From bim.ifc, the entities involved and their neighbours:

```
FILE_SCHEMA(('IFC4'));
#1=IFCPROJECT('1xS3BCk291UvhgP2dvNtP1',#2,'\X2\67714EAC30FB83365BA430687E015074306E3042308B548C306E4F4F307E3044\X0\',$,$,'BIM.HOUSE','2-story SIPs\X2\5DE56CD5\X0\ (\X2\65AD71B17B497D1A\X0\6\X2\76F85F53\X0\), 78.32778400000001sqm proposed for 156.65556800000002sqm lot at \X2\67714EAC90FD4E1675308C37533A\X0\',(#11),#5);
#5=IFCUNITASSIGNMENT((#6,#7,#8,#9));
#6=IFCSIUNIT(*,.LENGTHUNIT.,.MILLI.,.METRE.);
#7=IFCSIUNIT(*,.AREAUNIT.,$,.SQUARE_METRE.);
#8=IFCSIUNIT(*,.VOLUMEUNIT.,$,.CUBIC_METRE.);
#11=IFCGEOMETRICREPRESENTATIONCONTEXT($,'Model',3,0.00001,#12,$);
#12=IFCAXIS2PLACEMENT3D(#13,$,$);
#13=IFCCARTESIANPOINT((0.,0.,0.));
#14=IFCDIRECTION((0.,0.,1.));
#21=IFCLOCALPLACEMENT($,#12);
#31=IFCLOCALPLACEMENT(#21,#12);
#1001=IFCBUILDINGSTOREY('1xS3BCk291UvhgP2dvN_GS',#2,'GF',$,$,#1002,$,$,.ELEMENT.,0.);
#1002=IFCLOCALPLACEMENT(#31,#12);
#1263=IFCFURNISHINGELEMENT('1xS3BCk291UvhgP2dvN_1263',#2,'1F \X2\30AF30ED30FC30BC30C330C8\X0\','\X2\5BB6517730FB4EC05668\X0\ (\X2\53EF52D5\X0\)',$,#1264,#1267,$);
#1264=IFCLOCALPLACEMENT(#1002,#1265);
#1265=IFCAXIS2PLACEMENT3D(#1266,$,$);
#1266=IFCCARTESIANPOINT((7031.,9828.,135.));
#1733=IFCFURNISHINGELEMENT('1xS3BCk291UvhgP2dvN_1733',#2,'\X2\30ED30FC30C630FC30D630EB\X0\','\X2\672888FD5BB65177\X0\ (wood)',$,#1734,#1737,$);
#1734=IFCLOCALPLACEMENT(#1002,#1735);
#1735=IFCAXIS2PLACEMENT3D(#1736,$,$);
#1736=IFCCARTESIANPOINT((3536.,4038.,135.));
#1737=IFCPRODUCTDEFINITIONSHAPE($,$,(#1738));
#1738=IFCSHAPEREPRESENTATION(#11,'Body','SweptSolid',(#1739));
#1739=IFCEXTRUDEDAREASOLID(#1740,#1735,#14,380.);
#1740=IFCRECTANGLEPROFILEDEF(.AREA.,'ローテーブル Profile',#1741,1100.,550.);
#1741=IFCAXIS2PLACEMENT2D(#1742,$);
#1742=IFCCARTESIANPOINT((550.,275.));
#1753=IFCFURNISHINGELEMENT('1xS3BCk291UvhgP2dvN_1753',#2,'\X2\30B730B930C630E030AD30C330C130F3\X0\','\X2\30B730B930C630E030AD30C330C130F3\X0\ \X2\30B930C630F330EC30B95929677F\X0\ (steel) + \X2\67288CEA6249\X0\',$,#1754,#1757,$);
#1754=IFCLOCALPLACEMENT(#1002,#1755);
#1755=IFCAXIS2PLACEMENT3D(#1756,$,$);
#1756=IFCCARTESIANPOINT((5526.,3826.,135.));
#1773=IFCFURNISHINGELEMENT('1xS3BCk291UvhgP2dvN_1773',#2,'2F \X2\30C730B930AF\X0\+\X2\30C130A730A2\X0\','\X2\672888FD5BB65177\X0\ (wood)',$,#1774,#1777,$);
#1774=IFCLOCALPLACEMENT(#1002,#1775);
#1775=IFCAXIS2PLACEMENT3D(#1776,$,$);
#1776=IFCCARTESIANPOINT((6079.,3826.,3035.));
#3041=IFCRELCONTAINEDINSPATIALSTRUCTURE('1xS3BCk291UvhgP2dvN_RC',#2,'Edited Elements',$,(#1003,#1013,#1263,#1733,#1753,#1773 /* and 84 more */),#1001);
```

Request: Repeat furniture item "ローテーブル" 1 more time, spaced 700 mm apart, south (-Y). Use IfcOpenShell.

```python
import numpy as np
import ifcopenshell
import ifcopenshell.api.geometry
import ifcopenshell.api.root
import ifcopenshell.util.element
import ifcopenshell.util.placement
import ifcopenshell.util.unit

model = ifcopenshell.open("bim.ifc")
unit_scale = ifcopenshell.util.unit.calculate_unit_scale(model)


def reuse_history(source, copy):
    """copy_class also copies each property set's owner history, people and application; keep the originals."""
    for rel in copy.IsDefinedBy:
        if rel.is_a("IfcRelDefinesByProperties") and (history := rel.RelatingPropertyDefinition.OwnerHistory):
            rel.RelatingPropertyDefinition.OwnerHistory = source.OwnerHistory
            ifcopenshell.util.element.remove_deep2(model, history)


source = model.by_guid("1xS3BCk291UvhgP2dvN_1733")
base = ifcopenshell.util.placement.get_local_placement(source.ObjectPlacement)
step = np.array([0.0, -1.0, 0.0]) * 0.7 / unit_scale

for i in range(1, 2):
    copy = ifcopenshell.api.root.copy_class(model, product=source)
    copy.Representation = ifcopenshell.util.element.copy_deep(
        model, source.Representation, exclude=["IfcGeometricRepresentationContext", "IfcRepresentationMap"]
    )
    reuse_history(source, copy)
    matrix = base.copy()
    matrix[:3, 3] += i * step
    print("added at", matrix[:3, 3].round(3) + 0.0)
    ifcopenshell.api.geometry.edit_object_placement(model, product=copy, matrix=matrix, is_si=False)

model.write("bim_edited.ifc")
```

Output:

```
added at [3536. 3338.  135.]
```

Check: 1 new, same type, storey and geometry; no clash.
